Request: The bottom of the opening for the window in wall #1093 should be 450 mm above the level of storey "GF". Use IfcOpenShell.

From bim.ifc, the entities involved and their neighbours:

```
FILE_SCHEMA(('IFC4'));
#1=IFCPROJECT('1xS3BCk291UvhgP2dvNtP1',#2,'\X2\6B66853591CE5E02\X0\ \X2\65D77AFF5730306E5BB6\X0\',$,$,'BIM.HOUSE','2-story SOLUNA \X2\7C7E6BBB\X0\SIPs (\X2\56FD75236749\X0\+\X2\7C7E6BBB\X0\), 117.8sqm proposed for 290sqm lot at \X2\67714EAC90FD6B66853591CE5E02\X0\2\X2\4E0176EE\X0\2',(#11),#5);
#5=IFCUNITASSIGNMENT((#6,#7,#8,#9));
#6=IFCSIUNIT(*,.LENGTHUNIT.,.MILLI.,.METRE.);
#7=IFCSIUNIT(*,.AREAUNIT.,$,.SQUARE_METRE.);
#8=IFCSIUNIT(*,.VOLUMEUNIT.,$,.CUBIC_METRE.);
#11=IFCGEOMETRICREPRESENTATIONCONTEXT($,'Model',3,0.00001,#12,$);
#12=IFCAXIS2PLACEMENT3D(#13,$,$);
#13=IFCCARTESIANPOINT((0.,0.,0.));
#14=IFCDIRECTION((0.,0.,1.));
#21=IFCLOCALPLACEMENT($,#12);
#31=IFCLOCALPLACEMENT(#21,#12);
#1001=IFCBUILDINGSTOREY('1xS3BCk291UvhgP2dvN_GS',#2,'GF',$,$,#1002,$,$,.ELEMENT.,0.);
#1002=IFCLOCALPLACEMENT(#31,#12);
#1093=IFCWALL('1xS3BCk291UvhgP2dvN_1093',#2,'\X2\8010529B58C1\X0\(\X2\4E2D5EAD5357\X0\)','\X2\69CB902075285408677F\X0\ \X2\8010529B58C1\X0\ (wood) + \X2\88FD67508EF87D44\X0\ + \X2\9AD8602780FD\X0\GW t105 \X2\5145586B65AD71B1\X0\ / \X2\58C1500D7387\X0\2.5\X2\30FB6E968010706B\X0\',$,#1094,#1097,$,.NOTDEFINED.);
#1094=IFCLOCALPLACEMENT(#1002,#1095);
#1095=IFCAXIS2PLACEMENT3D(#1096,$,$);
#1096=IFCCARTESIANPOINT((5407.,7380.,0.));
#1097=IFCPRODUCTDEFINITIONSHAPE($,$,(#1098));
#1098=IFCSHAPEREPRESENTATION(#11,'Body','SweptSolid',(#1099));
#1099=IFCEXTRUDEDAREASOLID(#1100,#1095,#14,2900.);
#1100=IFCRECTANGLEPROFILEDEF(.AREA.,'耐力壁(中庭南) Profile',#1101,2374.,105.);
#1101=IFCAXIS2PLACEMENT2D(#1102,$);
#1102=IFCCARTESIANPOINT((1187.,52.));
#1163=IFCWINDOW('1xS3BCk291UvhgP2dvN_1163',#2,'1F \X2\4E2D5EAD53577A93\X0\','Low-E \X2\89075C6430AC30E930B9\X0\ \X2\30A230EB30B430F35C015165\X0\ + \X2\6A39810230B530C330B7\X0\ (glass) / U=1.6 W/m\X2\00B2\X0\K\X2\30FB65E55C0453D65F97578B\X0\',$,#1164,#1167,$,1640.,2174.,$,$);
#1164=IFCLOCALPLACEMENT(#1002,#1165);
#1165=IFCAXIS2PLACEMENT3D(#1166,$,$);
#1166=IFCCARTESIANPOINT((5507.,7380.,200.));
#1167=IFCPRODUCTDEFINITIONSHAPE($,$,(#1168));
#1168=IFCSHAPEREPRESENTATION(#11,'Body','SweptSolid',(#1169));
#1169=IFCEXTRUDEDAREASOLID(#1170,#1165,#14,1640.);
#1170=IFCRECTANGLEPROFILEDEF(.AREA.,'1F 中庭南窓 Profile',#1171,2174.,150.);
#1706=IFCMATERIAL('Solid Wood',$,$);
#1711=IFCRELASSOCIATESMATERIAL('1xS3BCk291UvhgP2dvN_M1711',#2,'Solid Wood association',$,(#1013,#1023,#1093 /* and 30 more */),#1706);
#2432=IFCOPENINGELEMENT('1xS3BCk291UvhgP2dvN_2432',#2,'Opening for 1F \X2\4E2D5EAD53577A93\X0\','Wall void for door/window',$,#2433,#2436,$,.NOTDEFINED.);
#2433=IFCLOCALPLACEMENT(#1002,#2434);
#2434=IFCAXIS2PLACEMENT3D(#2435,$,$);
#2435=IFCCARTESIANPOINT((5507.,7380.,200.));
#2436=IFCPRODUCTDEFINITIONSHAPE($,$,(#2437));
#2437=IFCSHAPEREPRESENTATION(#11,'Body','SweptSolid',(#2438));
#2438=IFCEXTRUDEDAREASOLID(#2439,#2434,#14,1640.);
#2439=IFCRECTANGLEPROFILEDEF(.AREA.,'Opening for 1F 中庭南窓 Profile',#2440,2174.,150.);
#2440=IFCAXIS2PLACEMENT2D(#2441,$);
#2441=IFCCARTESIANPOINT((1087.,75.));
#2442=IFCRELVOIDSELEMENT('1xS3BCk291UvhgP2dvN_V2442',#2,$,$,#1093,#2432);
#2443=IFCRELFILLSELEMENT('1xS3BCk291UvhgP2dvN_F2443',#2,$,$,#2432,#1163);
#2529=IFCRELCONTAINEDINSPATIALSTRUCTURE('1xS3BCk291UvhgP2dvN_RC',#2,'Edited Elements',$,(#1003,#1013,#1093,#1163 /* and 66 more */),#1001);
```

```python
import numpy as np
import ifcopenshell
import ifcopenshell.api.geometry
import ifcopenshell.geom
import ifcopenshell.util.element
import ifcopenshell.util.placement
import ifcopenshell.util.shape
import ifcopenshell.util.unit

model = ifcopenshell.open("bim.ifc")
unit_scale = ifcopenshell.util.unit.calculate_unit_scale(model)

window = model.by_id(1163)
opening = window.FillsVoids[0].RelatingOpeningElement
storey = ifcopenshell.util.element.get_container(window, ifc_class="IfcBuildingStorey")
level = ifcopenshell.util.placement.get_local_placement(storey.ObjectPlacement)[2, 3]

# The opening's origin need not be at the sill, so measure its lowest point.
shape = ifcopenshell.geom.create_shape(ifcopenshell.geom.settings(), opening)
bottom = ifcopenshell.util.shape.get_shape_bottom_elevation(shape, shape.geometry) / unit_scale
dz = level + 0.45 / unit_scale - bottom

shift = np.array([0.0, 0.0, dz])
# The window is not placed relative to its opening, so move both.
for product in (opening, window):
    matrix = ifcopenshell.util.placement.get_local_placement(product.ObjectPlacement)
    matrix[:3, 3] += shift
    ifcopenshell.api.geometry.edit_object_placement(model, product=product, matrix=matrix, is_si=False)

print(f"moved by {dz * unit_scale:+.3f} m")

model.write("bim-out.ifc")
```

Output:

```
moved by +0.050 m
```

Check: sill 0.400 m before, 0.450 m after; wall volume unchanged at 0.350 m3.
